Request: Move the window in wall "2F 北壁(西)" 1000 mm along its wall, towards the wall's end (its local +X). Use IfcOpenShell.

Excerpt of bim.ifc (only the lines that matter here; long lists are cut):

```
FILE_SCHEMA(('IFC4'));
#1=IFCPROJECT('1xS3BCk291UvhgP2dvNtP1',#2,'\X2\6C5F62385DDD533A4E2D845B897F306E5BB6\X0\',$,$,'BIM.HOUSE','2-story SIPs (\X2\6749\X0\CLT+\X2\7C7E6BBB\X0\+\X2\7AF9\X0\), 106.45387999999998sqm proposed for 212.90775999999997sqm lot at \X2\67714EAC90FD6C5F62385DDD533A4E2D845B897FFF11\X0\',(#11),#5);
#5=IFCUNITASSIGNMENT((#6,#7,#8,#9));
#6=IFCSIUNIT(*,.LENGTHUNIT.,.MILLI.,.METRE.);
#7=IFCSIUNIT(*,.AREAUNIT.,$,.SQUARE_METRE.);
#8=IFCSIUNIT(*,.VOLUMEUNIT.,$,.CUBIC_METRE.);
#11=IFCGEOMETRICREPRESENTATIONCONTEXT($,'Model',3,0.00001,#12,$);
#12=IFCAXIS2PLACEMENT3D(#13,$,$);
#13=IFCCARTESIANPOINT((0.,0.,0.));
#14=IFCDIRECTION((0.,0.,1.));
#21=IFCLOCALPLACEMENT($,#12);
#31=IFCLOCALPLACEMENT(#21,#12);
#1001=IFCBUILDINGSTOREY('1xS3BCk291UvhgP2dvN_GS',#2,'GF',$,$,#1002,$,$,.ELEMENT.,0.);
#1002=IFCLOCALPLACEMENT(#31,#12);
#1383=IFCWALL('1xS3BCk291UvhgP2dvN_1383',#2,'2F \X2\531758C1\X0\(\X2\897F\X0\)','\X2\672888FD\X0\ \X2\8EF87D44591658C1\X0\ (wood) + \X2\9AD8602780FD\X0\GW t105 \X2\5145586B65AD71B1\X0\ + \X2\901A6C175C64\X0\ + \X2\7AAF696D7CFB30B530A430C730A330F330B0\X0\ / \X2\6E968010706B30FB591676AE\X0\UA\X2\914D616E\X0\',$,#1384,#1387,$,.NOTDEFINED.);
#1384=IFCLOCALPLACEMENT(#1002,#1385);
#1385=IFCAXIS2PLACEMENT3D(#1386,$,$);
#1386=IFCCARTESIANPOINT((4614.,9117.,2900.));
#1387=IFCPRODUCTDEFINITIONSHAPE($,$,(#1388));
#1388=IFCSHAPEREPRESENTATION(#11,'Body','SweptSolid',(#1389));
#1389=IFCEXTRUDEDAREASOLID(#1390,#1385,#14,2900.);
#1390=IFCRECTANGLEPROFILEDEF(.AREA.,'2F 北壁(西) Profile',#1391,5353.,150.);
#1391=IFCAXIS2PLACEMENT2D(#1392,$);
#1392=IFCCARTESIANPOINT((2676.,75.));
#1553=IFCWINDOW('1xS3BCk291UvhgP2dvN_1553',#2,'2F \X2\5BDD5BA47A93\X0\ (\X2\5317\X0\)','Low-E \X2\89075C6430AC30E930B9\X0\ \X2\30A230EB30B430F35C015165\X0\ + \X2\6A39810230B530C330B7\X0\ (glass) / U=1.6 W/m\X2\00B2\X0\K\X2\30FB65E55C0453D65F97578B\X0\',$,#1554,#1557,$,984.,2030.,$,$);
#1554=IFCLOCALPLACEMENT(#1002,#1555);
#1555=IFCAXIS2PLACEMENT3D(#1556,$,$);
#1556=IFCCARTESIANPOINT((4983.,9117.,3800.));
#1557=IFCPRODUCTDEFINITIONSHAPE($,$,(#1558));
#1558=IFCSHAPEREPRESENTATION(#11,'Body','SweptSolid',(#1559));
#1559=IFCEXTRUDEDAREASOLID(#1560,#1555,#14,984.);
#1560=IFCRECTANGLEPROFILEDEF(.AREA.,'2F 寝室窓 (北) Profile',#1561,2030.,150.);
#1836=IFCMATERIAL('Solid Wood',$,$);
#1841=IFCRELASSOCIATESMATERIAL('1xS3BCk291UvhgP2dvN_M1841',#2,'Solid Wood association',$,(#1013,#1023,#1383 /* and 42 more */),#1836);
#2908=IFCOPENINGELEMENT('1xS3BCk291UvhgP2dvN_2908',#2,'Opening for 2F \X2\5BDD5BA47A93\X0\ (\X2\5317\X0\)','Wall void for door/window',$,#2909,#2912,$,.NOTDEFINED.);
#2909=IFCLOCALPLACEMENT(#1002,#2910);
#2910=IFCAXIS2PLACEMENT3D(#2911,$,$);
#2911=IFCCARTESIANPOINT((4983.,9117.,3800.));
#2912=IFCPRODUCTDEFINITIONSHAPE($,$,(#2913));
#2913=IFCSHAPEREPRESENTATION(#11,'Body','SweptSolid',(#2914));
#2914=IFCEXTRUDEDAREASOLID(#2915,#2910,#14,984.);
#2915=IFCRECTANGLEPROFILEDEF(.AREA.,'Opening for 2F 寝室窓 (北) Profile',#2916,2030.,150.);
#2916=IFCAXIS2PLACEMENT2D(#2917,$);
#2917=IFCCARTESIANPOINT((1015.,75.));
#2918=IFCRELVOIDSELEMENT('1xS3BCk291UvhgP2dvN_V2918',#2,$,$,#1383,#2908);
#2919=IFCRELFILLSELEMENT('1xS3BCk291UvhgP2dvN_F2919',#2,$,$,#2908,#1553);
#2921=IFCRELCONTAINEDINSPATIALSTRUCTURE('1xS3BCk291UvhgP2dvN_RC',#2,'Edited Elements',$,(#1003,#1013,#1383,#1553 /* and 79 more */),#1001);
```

```python
import ifcopenshell
import ifcopenshell.api.geometry
import ifcopenshell.util.placement

model = ifcopenshell.open("bim.ifc")

window = model.by_id(1553)
opening = window.FillsVoids[0].RelatingOpeningElement
wall = opening.VoidsElements[0].RelatingBuildingElement

wall_matrix = ifcopenshell.util.placement.get_local_placement(wall.ObjectPlacement)
shift = wall_matrix[:3, 0] * 1000.0
before = ifcopenshell.util.placement.get_local_placement(window.ObjectPlacement)[:3, 3].copy()

# The window is not placed relative to its opening, so move both.
for product in (opening, window):
    matrix = ifcopenshell.util.placement.get_local_placement(product.ObjectPlacement)
    matrix[:3, 3] += shift
    ifcopenshell.api.geometry.edit_object_placement(model, product=product, matrix=matrix, is_si=False)

after = ifcopenshell.util.placement.get_local_placement(window.ObjectPlacement)[:3, 3]
print("window moved by", (after - before).round(3) + 0.0)

model.write("bim_edited.ifc")
```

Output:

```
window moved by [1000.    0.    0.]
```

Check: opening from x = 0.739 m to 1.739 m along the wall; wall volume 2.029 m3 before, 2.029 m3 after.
